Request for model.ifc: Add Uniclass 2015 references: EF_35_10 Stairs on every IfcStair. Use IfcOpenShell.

First a look at what the model holds.

```python
import ifcopenshell

model = ifcopenshell.open("model.ifc")
print(model.schema)
print("classifications:", [c.Name for c in model.by_type("IfcClassification")])
for ifc_class in ("IfcDoor", "IfcRoof", "IfcStair", "IfcWall", "IfcWindow"):
    print(ifc_class, len(model.by_type(ifc_class)))
```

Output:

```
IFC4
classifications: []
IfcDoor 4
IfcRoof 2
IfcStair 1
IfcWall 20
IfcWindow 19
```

```python
import ifcopenshell
import ifcopenshell.api.classification

model = ifcopenshell.open("model.ifc")

system = ifcopenshell.api.classification.add_classification(model, classification="Uniclass 2015")

codes = {
    "IfcStair": ("EF_35_10", "Stairs"),
}
for ifc_class, (code, name) in codes.items():
    products = model.by_type(ifc_class)
    ifcopenshell.api.classification.add_reference(
        model, products=products, classification=system, identification=code, name=name
    )
    print(code, len(products))

model.write("model_rev.ifc")
```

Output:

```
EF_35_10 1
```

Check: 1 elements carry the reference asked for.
